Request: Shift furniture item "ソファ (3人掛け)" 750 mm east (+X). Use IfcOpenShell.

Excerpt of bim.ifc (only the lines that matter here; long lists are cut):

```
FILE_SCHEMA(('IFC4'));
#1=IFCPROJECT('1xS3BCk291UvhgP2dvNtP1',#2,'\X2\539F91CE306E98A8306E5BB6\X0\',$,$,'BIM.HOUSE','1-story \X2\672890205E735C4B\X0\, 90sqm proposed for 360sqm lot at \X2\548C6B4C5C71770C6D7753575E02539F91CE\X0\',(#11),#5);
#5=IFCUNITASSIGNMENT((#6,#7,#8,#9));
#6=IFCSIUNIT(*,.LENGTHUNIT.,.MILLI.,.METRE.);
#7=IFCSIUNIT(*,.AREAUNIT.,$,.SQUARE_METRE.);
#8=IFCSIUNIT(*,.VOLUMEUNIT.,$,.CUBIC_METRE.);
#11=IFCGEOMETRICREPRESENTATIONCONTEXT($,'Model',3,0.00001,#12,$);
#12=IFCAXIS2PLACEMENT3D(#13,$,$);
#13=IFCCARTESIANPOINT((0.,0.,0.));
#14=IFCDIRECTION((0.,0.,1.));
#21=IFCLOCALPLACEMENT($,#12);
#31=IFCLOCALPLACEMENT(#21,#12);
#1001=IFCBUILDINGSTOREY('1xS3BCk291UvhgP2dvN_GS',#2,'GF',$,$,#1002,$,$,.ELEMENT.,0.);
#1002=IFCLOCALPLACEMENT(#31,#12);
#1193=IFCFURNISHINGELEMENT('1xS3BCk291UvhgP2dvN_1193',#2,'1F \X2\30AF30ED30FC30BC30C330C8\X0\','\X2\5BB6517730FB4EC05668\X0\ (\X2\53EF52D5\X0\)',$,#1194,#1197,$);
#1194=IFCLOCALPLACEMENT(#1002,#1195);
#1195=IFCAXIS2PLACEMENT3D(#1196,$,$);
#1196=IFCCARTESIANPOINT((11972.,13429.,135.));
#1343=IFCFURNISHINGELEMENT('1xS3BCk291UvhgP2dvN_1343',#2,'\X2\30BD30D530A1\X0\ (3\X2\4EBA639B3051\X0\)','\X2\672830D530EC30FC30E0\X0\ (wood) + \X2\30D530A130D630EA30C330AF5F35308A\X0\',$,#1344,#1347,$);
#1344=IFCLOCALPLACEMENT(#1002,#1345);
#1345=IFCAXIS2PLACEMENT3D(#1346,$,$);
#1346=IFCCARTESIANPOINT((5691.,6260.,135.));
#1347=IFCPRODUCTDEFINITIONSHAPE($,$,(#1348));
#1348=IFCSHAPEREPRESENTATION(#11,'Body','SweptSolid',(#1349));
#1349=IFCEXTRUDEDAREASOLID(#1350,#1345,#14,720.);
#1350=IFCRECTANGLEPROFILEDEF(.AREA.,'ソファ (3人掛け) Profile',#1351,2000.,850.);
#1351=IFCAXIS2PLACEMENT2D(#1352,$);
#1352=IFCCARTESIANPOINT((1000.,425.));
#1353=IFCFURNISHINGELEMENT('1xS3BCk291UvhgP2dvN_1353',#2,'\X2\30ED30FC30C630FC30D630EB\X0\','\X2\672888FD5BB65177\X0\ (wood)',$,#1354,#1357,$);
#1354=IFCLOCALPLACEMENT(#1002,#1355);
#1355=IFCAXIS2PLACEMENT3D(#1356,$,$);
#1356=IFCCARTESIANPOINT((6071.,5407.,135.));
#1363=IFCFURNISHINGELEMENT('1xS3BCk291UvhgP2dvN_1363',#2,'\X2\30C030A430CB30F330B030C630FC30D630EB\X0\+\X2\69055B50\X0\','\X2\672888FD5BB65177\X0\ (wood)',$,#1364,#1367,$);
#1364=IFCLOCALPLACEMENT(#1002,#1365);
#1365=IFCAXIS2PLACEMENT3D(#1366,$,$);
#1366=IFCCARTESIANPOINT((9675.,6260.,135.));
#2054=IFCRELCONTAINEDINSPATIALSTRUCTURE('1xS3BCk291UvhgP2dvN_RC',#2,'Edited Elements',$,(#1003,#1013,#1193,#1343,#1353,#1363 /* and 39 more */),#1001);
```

```python
import ifcopenshell
import ifcopenshell.api.geometry
import ifcopenshell.util.placement

model = ifcopenshell.open("bim.ifc")

item = model.by_guid("1xS3BCk291UvhgP2dvN_1343")
matrix = ifcopenshell.util.placement.get_local_placement(item.ObjectPlacement)
matrix[0, 3] += 750.0
ifcopenshell.api.geometry.edit_object_placement(model, product=item, matrix=matrix, is_si=False)

print(ifcopenshell.util.placement.get_local_placement(item.ObjectPlacement).round(3) + 0.0)

model.write("bim_edited.ifc")
```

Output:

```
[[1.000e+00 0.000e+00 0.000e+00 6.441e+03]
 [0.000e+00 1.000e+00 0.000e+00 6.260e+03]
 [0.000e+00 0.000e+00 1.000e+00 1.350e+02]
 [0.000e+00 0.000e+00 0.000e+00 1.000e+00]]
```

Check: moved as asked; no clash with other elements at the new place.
